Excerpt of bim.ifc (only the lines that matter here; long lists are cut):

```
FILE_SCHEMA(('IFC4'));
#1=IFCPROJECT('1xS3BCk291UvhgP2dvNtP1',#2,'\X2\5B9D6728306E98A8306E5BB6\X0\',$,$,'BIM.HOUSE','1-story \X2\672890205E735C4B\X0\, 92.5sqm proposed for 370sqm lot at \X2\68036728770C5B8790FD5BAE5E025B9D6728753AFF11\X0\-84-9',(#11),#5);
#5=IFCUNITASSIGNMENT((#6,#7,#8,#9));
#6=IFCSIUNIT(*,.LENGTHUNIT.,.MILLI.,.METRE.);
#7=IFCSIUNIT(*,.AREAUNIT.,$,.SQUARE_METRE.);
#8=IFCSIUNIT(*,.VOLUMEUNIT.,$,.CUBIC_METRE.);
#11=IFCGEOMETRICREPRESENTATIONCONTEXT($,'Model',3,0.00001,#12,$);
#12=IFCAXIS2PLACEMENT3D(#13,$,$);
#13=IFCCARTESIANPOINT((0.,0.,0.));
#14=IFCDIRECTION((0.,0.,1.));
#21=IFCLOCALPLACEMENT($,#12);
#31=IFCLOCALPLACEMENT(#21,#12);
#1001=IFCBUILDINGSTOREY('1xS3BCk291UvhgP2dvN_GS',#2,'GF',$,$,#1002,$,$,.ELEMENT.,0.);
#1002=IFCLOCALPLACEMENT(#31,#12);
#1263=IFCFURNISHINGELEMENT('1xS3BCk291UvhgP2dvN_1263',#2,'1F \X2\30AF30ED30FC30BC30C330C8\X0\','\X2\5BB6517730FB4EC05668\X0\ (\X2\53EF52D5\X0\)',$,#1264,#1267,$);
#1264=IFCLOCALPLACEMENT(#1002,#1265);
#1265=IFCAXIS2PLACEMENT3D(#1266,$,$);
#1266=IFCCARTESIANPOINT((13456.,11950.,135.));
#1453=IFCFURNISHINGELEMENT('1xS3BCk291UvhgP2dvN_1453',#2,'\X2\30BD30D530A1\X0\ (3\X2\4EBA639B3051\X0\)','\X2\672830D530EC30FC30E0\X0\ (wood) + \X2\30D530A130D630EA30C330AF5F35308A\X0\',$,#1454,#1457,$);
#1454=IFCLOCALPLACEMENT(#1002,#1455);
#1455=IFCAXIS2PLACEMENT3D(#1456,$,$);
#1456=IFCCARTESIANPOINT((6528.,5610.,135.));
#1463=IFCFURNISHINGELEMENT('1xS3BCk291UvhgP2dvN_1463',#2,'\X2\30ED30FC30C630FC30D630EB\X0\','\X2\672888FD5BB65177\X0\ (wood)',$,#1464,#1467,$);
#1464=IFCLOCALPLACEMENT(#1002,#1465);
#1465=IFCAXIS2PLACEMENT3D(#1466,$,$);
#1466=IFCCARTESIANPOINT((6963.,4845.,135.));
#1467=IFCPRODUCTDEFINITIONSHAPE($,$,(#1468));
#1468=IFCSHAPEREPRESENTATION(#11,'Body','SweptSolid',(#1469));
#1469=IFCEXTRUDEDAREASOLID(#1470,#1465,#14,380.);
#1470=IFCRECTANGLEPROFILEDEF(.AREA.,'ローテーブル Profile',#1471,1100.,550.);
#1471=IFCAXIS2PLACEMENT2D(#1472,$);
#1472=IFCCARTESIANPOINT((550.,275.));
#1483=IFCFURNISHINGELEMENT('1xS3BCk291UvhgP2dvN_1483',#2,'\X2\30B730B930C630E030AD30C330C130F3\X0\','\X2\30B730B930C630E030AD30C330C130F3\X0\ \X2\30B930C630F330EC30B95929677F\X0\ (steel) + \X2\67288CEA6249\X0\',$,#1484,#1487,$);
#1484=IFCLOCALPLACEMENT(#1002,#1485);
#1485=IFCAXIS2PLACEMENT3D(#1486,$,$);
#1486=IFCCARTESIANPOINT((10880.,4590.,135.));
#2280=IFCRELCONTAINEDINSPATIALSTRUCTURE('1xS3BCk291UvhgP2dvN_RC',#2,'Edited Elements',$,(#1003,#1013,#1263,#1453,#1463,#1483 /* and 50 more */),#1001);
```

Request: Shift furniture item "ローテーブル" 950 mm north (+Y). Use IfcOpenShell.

```python
import ifcopenshell
import ifcopenshell.api.geometry
import ifcopenshell.util.placement
import ifcopenshell.util.unit

model = ifcopenshell.open("bim.ifc")
unit_scale = ifcopenshell.util.unit.calculate_unit_scale(model)

item = model.by_guid("1xS3BCk291UvhgP2dvN_1463")
matrix = ifcopenshell.util.placement.get_local_placement(item.ObjectPlacement)
matrix[1, 3] += 0.95 / unit_scale
ifcopenshell.api.geometry.edit_object_placement(model, product=item, matrix=matrix, is_si=False)

print(ifcopenshell.util.placement.get_local_placement(item.ObjectPlacement).round(3) + 0.0)

model.write("bim_v2.ifc")
```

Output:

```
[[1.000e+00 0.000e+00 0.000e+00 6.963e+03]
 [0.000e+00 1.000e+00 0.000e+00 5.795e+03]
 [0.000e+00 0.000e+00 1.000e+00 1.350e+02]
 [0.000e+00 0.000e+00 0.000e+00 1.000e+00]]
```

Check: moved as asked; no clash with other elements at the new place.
